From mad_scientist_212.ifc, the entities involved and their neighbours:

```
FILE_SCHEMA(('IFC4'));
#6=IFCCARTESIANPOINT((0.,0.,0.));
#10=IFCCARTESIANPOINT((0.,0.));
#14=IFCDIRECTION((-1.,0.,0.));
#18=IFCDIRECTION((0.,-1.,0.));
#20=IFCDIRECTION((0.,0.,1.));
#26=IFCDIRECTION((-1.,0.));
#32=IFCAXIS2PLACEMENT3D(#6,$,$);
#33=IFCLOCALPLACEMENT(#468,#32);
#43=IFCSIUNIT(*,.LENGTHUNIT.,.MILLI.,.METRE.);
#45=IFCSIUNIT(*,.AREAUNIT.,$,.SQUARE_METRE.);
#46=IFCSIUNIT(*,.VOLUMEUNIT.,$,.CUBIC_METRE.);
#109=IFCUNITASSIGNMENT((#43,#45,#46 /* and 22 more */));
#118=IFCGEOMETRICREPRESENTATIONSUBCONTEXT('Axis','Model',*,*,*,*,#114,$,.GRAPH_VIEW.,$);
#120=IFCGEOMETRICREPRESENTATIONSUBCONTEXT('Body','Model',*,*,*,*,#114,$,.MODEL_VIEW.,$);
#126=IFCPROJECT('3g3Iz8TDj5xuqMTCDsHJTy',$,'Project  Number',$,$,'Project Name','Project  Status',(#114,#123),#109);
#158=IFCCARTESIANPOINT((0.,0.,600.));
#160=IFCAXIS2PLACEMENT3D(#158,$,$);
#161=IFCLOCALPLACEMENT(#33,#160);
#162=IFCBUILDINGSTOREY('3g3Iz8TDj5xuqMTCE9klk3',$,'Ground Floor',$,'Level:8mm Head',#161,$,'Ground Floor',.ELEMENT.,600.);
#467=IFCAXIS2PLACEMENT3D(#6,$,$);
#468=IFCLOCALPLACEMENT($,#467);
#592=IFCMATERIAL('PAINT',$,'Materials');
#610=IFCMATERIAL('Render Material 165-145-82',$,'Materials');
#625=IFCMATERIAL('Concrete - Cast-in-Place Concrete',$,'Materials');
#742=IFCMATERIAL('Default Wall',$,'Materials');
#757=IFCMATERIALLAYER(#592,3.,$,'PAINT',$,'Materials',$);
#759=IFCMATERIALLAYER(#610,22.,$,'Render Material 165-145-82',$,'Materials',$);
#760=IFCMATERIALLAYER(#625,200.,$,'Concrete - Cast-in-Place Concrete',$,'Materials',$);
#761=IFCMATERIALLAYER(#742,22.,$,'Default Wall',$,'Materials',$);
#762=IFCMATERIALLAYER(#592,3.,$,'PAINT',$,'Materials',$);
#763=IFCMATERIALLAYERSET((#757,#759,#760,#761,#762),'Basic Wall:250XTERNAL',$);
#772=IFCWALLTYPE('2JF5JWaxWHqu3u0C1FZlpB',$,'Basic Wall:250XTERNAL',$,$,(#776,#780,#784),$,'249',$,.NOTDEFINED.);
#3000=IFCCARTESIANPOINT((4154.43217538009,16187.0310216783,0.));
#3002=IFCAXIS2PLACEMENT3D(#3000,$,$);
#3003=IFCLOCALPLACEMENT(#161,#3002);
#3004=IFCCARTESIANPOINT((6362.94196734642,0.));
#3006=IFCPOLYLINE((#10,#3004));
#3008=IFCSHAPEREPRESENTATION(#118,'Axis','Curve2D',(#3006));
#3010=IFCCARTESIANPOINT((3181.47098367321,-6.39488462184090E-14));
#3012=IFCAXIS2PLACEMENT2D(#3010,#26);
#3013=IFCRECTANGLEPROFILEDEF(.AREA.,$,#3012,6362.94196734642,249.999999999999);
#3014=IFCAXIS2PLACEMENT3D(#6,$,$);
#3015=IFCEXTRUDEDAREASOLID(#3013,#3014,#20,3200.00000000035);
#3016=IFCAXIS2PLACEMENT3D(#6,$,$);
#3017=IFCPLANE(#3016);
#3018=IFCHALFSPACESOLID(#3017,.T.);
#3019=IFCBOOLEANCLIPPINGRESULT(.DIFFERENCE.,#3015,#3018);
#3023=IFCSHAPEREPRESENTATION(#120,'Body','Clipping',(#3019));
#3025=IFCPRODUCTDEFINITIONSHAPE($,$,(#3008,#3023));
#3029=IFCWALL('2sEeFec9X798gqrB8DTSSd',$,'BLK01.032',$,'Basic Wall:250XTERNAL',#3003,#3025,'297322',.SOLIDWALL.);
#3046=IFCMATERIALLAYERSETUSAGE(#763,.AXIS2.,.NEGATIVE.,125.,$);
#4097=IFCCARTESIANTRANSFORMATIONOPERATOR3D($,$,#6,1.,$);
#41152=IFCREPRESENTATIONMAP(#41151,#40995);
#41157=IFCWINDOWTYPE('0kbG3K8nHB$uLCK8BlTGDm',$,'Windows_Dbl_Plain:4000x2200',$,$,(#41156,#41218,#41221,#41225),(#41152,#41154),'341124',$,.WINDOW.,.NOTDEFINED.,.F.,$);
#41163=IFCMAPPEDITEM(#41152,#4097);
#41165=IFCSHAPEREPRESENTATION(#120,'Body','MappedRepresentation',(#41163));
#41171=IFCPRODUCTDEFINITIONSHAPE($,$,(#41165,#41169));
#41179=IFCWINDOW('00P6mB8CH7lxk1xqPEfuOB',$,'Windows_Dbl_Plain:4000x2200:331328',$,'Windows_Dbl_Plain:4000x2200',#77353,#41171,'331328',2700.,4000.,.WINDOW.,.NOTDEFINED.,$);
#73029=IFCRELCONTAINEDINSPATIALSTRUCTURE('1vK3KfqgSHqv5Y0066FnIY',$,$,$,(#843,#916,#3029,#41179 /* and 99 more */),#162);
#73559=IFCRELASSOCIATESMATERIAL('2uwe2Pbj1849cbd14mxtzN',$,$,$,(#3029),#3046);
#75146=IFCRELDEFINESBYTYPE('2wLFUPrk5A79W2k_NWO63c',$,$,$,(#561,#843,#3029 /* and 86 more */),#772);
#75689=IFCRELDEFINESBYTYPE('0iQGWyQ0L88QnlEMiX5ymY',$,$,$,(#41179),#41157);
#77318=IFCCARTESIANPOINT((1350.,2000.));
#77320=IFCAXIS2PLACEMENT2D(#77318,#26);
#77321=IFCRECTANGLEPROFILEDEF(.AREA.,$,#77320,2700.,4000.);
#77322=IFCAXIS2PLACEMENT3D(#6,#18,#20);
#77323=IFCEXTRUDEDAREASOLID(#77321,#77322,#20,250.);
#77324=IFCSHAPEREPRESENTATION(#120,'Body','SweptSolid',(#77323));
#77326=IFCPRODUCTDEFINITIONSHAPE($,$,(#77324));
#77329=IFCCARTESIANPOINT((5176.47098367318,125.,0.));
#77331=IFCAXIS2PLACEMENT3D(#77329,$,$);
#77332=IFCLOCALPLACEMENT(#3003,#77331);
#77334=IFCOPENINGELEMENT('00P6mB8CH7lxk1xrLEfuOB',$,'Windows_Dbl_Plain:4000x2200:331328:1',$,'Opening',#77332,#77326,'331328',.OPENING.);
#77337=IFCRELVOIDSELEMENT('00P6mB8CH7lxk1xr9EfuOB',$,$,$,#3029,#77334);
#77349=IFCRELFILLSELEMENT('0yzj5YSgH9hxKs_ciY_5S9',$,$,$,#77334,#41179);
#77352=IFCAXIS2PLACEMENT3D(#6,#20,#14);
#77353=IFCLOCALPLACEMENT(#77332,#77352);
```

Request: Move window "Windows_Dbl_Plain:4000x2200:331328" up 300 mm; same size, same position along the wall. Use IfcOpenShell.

```python
import numpy as np
import ifcopenshell
import ifcopenshell.api.geometry
import ifcopenshell.util.placement
import ifcopenshell.util.unit

model = ifcopenshell.open("mad_scientist_212.ifc")
unit_scale = ifcopenshell.util.unit.calculate_unit_scale(model)

window = model.by_guid("00P6mB8CH7lxk1xqPEfuOB")
opening = window.FillsVoids[0].RelatingOpeningElement
dz = 300.0

shift = np.array([0.0, 0.0, dz])
# The window is placed relative to its opening, so it follows when the opening moves.
matrix = ifcopenshell.util.placement.get_local_placement(opening.ObjectPlacement)
matrix[:3, 3] += shift
ifcopenshell.api.geometry.edit_object_placement(
    model, product=opening, matrix=matrix, is_si=False, should_transform_children=True
)

print(f"moved by {dz * unit_scale:+.3f} m")

model.write("mad_scientist_212_rev.ifc")
```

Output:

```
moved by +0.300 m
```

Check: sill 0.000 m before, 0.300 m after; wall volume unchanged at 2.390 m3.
